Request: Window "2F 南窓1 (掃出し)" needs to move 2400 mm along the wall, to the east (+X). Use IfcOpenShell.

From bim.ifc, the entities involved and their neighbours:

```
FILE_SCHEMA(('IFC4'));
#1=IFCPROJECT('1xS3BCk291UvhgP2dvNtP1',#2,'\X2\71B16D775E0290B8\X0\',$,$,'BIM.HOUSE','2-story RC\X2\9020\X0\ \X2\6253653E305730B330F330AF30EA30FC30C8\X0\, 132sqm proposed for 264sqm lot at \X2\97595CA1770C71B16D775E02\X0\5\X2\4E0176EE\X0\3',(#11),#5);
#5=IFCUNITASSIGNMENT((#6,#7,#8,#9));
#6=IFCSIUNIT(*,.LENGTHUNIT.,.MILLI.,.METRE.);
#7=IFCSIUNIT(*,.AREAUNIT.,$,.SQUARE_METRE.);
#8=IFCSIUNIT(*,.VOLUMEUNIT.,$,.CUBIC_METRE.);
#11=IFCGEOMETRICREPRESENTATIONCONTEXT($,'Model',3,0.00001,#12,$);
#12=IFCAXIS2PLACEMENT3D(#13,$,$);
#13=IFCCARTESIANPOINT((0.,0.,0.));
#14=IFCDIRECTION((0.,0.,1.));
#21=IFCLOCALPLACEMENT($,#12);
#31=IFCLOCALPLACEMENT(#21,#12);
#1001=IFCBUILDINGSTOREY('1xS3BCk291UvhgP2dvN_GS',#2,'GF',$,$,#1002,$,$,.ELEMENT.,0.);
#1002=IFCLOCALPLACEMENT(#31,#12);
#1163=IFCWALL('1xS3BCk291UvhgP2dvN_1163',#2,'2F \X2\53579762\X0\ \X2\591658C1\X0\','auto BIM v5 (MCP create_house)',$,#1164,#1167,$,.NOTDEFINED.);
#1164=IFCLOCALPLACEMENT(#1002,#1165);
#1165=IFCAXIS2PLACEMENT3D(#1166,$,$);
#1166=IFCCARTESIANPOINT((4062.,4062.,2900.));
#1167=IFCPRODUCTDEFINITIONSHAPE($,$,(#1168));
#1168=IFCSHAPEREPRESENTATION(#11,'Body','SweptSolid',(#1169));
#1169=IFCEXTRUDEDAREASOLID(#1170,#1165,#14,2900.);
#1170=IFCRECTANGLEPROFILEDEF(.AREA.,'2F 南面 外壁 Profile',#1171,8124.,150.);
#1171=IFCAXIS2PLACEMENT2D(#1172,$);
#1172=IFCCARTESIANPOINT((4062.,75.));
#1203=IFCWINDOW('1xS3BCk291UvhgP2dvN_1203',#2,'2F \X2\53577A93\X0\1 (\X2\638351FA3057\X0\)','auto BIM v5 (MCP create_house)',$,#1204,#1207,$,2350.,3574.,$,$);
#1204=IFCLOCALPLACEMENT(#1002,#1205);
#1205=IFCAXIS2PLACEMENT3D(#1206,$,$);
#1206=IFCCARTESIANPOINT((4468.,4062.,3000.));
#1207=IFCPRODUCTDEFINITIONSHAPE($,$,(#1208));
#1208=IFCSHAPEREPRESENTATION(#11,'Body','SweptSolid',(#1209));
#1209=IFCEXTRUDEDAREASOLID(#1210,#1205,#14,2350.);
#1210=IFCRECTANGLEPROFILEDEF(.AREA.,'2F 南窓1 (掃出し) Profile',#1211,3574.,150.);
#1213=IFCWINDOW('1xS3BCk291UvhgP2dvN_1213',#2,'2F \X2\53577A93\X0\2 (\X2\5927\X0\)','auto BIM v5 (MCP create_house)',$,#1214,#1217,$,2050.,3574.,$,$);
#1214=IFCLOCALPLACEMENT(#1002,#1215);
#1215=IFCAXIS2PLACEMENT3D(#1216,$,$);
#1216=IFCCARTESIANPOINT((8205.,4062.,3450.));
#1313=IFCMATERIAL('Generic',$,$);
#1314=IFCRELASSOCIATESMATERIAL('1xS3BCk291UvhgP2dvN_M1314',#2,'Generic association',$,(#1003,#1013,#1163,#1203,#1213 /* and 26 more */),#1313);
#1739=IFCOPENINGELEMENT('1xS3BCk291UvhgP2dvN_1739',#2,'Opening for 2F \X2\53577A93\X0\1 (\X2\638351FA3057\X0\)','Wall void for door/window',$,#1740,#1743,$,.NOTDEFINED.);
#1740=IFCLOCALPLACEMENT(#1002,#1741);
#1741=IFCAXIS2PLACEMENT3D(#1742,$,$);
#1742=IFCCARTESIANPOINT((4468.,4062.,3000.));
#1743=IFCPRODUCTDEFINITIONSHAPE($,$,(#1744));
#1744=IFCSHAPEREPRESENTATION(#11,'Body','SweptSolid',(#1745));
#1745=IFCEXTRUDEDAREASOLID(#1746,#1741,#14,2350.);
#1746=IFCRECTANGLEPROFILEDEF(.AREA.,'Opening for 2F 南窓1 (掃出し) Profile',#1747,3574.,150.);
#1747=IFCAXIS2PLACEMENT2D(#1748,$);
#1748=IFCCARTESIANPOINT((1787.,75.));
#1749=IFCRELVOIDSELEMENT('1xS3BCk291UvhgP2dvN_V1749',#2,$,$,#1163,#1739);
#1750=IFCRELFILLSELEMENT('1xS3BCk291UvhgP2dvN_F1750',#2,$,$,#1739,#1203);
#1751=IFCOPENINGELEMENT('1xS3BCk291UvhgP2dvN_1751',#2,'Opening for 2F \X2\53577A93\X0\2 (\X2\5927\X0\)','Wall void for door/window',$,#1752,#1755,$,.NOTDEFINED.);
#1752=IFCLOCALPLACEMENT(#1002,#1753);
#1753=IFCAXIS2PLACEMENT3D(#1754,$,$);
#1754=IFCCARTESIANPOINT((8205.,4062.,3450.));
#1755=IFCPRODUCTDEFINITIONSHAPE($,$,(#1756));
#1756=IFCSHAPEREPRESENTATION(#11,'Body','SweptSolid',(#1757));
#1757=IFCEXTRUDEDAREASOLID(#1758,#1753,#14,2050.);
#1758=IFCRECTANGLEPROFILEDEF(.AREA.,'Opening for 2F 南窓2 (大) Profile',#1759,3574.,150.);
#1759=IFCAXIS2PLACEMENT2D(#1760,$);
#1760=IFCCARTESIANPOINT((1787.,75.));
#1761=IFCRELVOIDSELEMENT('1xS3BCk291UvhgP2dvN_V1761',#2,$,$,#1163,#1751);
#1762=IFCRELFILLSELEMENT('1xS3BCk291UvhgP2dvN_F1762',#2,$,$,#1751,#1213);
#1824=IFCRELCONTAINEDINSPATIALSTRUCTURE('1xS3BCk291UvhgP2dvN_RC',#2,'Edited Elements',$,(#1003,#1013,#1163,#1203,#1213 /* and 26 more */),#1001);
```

```python
import ifcopenshell
import ifcopenshell.api.geometry
import ifcopenshell.util.placement
import ifcopenshell.util.unit

model = ifcopenshell.open("bim.ifc")
unit_scale = ifcopenshell.util.unit.calculate_unit_scale(model)

window = model.by_id(1203)
opening = window.FillsVoids[0].RelatingOpeningElement
wall = opening.VoidsElements[0].RelatingBuildingElement

wall_matrix = ifcopenshell.util.placement.get_local_placement(wall.ObjectPlacement)
shift = wall_matrix[:3, 0] * 2.4 / unit_scale
before = ifcopenshell.util.placement.get_local_placement(window.ObjectPlacement)[:3, 3].copy()

# The window is not placed relative to its opening, so move both.
for product in (opening, window):
    matrix = ifcopenshell.util.placement.get_local_placement(product.ObjectPlacement)
    matrix[:3, 3] += shift
    ifcopenshell.api.geometry.edit_object_placement(model, product=product, matrix=matrix, is_si=False)

after = ifcopenshell.util.placement.get_local_placement(window.ObjectPlacement)[:3, 3]
print("window moved by", (after - before).round(3) + 0.0)

model.write("bim_edited.ifc")
```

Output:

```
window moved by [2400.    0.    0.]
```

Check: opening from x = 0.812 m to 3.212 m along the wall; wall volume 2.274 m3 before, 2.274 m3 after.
